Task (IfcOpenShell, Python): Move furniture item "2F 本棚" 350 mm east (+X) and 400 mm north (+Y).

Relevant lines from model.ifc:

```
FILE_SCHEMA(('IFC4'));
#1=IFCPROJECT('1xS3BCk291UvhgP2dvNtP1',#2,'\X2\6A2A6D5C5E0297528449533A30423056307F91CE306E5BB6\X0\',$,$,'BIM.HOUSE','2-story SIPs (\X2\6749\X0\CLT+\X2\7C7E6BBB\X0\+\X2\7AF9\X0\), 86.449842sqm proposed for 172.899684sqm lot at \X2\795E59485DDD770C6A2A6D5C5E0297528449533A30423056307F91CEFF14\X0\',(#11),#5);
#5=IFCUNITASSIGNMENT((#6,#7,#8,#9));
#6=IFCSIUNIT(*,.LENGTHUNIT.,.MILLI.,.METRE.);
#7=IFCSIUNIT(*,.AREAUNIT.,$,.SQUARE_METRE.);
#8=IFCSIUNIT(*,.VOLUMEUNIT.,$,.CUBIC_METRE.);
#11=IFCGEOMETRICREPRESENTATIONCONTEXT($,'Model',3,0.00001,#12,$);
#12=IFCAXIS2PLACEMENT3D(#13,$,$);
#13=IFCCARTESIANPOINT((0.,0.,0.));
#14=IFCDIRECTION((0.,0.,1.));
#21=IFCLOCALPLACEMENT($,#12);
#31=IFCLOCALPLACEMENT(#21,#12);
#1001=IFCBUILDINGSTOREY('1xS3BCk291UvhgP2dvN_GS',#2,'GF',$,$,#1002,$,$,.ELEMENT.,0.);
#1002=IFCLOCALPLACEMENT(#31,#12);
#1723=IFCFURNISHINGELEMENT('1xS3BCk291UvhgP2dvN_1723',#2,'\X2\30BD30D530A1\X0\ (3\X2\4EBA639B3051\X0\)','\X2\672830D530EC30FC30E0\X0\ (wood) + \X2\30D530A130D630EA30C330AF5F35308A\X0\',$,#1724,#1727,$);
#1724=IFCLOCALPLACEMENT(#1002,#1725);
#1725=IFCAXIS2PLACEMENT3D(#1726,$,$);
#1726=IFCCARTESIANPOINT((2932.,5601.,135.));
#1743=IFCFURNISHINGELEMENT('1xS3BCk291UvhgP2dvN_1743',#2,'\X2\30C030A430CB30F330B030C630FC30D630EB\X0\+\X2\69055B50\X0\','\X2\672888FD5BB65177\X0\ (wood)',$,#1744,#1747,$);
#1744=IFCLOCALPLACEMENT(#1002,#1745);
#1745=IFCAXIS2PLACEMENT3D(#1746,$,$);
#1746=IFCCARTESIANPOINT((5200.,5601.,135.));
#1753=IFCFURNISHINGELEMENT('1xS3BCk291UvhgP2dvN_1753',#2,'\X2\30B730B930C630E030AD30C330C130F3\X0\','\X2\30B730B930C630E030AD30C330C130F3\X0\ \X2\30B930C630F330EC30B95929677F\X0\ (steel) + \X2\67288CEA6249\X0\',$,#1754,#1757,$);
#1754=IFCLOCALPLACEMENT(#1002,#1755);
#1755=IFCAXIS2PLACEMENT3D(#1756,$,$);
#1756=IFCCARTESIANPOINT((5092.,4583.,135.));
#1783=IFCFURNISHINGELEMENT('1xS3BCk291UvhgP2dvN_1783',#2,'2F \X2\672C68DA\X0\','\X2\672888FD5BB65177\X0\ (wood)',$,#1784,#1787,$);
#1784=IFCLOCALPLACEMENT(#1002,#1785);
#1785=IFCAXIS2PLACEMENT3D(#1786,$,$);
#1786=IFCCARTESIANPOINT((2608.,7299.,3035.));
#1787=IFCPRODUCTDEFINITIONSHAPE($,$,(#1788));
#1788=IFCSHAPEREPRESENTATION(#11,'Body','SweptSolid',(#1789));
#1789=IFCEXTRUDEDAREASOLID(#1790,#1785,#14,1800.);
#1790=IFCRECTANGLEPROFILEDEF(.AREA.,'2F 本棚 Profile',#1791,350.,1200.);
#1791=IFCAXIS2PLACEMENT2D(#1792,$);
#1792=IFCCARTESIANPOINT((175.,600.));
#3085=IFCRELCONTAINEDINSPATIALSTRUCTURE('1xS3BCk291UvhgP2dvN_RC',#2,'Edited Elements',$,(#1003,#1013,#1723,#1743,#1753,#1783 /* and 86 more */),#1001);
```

```python
import ifcopenshell
import ifcopenshell.api.geometry
import ifcopenshell.util.placement
import ifcopenshell.util.unit

model = ifcopenshell.open("model.ifc")
unit_scale = ifcopenshell.util.unit.calculate_unit_scale(model)

item = model.by_guid("1xS3BCk291UvhgP2dvN_1783")
matrix = ifcopenshell.util.placement.get_local_placement(item.ObjectPlacement)
matrix[0, 3] += 0.35 / unit_scale
matrix[1, 3] += 0.4 / unit_scale
ifcopenshell.api.geometry.edit_object_placement(model, product=item, matrix=matrix, is_si=False)

print(ifcopenshell.util.placement.get_local_placement(item.ObjectPlacement).round(3) + 0.0)

model.write("model_v2.ifc")
```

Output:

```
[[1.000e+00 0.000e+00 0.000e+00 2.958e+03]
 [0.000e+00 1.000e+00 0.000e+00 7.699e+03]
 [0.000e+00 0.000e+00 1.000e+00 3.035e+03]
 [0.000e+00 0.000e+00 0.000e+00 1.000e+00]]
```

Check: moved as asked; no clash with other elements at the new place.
